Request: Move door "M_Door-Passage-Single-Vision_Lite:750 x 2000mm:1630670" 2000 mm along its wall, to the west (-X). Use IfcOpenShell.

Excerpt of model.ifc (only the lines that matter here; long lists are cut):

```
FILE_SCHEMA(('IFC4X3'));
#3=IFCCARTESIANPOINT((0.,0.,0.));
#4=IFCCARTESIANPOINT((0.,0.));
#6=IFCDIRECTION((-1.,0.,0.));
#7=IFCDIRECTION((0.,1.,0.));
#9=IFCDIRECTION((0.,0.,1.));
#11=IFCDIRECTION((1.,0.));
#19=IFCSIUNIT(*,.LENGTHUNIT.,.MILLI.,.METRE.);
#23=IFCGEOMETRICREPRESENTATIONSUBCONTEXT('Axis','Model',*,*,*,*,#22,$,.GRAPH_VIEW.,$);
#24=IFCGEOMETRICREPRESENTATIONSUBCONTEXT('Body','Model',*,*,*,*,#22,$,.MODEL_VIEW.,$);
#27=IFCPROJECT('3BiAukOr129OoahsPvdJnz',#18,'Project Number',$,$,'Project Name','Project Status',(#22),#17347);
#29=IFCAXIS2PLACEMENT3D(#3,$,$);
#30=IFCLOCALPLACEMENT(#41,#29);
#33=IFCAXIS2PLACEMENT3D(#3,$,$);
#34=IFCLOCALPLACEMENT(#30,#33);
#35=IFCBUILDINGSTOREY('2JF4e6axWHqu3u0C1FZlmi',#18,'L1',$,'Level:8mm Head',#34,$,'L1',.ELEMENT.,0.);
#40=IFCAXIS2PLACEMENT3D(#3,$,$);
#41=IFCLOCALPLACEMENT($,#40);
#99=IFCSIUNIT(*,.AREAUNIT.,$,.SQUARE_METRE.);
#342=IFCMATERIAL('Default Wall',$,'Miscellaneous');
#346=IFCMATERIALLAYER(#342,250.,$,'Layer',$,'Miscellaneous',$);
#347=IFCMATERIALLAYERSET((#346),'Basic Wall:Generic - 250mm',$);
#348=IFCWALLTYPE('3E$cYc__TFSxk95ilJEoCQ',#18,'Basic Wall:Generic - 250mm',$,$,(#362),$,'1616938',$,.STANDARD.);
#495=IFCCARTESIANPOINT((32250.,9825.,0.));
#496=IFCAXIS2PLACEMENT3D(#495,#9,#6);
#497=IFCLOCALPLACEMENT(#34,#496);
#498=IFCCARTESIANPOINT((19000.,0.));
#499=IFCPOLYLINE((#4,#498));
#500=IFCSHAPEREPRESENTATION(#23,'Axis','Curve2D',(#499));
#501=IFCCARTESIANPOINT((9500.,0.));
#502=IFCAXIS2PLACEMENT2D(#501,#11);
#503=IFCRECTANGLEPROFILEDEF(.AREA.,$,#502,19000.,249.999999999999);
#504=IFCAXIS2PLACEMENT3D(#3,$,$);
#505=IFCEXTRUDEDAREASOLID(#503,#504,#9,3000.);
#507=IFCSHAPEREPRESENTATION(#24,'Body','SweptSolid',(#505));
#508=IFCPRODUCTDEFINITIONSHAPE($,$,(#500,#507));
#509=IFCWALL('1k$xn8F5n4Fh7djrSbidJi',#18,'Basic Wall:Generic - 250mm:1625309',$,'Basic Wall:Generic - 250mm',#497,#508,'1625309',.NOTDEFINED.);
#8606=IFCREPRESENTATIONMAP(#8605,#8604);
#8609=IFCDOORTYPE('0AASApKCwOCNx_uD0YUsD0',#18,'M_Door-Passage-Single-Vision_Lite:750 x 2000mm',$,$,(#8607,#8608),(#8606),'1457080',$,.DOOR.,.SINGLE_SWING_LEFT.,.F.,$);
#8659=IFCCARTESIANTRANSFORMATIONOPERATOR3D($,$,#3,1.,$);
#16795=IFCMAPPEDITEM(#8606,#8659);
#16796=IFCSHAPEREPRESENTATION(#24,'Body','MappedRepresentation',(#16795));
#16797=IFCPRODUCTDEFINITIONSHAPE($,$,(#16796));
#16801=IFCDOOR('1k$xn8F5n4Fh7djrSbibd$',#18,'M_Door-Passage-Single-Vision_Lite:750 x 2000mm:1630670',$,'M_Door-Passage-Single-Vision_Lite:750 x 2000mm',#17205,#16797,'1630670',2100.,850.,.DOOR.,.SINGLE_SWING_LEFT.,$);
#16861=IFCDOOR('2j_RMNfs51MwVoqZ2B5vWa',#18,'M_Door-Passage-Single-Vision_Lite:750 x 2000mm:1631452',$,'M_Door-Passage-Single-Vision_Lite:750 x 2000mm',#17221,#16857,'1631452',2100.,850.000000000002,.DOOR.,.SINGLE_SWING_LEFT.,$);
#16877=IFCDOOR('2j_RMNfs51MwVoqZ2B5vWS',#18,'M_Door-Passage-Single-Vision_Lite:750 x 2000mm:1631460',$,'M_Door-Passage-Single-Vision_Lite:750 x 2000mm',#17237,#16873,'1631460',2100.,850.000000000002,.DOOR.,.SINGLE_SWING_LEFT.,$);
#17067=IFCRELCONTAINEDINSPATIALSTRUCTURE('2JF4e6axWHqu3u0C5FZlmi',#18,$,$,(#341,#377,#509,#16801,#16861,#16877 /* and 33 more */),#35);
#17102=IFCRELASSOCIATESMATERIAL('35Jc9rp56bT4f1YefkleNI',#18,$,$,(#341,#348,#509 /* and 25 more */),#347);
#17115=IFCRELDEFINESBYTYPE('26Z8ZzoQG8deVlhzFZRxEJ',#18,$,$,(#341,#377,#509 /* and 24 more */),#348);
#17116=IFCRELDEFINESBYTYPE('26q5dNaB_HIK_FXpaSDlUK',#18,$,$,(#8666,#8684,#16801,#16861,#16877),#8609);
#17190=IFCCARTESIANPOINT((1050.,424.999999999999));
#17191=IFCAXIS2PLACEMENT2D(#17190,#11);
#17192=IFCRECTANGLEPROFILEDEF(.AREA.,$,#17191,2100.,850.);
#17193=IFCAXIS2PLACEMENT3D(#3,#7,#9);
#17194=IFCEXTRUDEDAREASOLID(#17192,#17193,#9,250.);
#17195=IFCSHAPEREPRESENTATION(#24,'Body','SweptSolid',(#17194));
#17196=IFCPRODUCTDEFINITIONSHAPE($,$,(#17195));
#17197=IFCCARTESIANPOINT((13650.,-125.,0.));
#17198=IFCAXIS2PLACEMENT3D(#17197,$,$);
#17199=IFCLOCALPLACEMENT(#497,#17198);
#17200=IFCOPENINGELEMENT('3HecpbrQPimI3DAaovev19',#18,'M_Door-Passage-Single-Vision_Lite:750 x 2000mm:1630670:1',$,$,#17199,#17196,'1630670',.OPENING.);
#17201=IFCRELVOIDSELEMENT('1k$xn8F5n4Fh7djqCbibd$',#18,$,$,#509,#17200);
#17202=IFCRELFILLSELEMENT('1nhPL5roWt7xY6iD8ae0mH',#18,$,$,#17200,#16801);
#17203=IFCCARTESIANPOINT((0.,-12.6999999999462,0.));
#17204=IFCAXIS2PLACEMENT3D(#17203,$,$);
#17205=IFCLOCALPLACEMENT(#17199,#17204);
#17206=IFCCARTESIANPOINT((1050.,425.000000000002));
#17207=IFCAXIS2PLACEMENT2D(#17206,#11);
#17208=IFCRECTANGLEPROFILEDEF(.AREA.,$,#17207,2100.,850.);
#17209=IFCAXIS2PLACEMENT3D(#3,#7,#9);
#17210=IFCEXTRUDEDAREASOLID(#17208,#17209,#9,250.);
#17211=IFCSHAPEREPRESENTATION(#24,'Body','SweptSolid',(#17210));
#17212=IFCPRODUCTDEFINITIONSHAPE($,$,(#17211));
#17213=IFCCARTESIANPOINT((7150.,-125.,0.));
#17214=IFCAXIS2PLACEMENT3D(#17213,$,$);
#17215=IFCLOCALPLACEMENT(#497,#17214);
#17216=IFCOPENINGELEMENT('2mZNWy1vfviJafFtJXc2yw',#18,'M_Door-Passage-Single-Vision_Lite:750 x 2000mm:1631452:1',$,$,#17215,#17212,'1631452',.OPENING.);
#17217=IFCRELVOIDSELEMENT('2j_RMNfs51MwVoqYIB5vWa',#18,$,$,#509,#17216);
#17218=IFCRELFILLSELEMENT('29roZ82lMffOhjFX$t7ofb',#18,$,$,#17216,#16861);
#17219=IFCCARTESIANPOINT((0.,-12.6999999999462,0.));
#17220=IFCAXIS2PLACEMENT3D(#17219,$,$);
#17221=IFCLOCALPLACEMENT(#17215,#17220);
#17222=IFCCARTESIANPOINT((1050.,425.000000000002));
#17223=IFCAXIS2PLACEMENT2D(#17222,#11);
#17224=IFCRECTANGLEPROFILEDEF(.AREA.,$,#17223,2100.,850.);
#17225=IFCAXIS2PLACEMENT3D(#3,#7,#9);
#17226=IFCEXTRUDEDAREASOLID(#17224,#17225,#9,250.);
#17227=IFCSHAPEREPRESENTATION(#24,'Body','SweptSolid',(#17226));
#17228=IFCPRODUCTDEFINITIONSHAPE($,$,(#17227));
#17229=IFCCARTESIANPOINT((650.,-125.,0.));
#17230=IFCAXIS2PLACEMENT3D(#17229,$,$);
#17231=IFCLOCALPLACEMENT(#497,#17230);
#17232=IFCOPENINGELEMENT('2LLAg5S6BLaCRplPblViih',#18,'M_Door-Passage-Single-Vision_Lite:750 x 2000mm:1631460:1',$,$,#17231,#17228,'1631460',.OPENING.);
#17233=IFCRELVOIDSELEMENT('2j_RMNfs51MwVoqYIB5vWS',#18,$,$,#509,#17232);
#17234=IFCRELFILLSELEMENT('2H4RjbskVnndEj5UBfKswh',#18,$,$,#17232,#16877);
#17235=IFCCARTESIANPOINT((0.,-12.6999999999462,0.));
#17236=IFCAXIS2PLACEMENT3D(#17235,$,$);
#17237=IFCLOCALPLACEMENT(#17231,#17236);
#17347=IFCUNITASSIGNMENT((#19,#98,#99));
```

```python
import ifcopenshell
import ifcopenshell.api.geometry
import ifcopenshell.util.placement

model = ifcopenshell.open("model.ifc")

door = model.by_guid("1k$xn8F5n4Fh7djrSbibd$")
opening = door.FillsVoids[0].RelatingOpeningElement
wall = opening.VoidsElements[0].RelatingBuildingElement

wall_matrix = ifcopenshell.util.placement.get_local_placement(wall.ObjectPlacement)
shift = wall_matrix[:3, 0] * 2000.0
before = ifcopenshell.util.placement.get_local_placement(door.ObjectPlacement)[:3, 3].copy()

# The door is placed relative to its opening, so it follows when the opening moves.
matrix = ifcopenshell.util.placement.get_local_placement(opening.ObjectPlacement)
matrix[:3, 3] += shift
ifcopenshell.api.geometry.edit_object_placement(
    model, product=opening, matrix=matrix, is_si=False, should_transform_children=True
)

after = ifcopenshell.util.placement.get_local_placement(door.ObjectPlacement)[:3, 3]
print("door moved by", (after - before).round(3) + 0.0)

model.write("model_updated.ifc")
```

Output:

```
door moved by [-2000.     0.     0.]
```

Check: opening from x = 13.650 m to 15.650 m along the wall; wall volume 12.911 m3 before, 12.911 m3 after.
